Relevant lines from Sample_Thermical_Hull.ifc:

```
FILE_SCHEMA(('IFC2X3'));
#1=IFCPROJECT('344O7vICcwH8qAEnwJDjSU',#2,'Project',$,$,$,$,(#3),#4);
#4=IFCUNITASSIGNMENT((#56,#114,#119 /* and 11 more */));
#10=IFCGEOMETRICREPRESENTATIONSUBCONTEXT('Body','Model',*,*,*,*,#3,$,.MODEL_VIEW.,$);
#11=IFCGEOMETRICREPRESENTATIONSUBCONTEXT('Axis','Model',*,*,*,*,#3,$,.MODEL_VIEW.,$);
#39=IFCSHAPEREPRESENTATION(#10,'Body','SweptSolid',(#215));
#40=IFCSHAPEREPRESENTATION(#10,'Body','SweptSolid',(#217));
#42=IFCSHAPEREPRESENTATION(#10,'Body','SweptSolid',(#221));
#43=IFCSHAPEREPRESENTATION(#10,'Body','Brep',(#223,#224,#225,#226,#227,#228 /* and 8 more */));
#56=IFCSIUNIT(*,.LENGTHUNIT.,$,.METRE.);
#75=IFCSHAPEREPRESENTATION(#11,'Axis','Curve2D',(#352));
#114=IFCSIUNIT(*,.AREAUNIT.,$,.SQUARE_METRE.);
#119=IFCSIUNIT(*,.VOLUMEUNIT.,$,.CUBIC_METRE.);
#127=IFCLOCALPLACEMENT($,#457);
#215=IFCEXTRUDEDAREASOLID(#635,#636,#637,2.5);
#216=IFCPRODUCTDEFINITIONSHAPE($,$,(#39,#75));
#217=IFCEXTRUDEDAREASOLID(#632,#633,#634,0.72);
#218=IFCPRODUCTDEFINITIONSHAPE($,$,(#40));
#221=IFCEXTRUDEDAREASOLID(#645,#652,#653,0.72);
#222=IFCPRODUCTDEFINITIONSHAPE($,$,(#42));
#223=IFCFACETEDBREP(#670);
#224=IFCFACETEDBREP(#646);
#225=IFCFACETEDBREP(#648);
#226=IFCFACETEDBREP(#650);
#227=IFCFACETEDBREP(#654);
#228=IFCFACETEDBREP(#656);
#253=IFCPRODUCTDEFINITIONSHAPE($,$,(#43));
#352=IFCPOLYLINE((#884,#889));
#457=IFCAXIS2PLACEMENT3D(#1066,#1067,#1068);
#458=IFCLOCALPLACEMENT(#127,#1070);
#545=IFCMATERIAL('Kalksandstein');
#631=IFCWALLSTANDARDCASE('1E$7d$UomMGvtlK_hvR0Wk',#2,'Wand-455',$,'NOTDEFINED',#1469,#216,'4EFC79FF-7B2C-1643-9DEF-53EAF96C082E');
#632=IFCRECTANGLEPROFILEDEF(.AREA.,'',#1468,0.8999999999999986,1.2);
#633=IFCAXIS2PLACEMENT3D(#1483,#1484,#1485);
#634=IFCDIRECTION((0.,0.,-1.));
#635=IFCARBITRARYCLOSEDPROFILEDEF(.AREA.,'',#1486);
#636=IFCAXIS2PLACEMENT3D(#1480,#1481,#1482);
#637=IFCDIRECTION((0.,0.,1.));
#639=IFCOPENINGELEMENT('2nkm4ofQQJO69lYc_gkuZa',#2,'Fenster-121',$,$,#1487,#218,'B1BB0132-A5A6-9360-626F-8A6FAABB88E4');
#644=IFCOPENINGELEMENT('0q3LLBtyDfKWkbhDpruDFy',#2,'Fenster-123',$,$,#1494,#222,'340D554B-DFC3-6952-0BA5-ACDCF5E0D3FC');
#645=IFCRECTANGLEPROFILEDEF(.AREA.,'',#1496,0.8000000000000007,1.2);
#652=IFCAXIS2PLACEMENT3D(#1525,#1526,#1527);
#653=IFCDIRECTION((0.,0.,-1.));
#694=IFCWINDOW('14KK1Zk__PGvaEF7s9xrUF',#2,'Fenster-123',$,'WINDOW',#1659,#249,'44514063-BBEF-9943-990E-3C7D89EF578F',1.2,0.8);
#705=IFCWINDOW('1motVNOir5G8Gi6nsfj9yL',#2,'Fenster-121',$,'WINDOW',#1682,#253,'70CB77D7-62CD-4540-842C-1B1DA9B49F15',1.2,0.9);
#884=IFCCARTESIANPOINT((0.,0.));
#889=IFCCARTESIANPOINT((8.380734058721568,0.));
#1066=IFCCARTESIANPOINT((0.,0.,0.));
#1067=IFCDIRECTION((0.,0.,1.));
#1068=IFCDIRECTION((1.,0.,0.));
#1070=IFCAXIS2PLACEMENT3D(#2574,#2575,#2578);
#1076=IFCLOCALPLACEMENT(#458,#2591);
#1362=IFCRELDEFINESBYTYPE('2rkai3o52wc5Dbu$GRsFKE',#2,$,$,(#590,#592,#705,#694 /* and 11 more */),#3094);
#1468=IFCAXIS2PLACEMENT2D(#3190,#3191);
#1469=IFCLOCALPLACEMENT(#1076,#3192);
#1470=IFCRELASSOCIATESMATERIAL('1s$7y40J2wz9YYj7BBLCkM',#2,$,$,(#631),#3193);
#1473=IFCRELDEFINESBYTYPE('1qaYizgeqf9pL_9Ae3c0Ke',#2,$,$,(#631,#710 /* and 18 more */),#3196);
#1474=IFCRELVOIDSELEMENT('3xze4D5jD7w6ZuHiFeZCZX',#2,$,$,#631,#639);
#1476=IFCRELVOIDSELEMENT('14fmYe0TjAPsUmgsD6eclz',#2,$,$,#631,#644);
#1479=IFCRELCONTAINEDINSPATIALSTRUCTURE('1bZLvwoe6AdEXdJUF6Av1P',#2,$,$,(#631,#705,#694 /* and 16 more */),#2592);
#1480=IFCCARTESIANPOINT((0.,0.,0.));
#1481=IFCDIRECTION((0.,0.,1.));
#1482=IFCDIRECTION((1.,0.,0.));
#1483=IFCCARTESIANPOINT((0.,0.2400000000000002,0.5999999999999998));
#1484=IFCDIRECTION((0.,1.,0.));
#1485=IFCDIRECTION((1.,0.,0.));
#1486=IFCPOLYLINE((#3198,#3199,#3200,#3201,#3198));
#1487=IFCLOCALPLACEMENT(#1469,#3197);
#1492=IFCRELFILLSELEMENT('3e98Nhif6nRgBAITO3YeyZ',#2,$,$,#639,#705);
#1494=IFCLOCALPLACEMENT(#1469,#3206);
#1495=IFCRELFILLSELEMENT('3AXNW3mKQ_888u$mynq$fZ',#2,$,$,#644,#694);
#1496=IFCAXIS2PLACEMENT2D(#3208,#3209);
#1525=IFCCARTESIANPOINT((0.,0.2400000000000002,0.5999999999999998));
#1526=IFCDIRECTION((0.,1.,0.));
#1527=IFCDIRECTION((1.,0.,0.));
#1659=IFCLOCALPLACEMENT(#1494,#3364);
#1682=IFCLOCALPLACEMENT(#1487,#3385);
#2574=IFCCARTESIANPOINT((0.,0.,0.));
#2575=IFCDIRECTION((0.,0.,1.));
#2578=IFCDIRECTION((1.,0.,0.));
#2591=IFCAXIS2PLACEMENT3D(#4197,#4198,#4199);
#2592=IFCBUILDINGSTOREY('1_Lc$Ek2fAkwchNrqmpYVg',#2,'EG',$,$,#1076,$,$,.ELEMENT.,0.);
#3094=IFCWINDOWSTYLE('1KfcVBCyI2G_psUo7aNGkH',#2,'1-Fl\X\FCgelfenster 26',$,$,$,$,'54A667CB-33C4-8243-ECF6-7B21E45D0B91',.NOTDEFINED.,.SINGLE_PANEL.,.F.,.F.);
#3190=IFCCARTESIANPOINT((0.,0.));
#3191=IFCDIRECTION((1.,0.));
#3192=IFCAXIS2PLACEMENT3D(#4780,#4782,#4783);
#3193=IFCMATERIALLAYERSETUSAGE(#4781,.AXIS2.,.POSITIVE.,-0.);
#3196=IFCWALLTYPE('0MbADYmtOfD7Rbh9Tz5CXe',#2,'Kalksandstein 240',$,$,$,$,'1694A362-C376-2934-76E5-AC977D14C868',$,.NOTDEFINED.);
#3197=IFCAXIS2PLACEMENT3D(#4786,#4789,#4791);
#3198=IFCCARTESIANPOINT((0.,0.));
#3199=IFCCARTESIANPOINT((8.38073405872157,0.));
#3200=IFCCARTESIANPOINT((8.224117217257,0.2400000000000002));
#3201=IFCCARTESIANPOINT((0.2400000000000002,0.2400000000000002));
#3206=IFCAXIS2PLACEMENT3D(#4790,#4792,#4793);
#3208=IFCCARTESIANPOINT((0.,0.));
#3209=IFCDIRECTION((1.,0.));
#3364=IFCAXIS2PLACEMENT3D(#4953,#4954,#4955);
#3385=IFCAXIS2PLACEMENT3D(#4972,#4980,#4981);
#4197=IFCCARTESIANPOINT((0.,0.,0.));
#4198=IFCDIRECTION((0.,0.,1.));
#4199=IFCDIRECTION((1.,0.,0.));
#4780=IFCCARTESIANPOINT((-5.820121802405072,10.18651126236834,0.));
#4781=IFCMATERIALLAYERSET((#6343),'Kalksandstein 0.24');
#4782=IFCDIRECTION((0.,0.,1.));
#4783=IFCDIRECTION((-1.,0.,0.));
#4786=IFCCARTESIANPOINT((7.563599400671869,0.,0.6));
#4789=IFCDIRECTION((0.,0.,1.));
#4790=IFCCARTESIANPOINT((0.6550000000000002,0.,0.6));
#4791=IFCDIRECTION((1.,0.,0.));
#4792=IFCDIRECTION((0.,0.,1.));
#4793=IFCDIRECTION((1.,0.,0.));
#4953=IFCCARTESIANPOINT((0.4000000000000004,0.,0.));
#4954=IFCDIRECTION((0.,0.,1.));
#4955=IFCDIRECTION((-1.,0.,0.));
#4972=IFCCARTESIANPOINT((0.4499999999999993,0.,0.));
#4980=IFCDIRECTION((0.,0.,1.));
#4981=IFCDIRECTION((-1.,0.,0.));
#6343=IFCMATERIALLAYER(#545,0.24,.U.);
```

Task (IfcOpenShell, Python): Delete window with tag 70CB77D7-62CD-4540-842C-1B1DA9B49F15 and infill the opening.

```python
import ifcopenshell
import ifcopenshell.api.feature
import ifcopenshell.api.root
import ifcopenshell.geom
import ifcopenshell.util.shape

model = ifcopenshell.open("Sample_Thermical_Hull.ifc")
settings = ifcopenshell.geom.settings()


def volume(element):
    """Net volume in cubic metres, openings subtracted."""
    shape = ifcopenshell.geom.create_shape(settings, element)
    return ifcopenshell.util.shape.get_volume(shape.geometry)


window = model.by_guid("1motVNOir5G8Gi6nsfj9yL")
opening = window.FillsVoids[0].RelatingOpeningElement
wall = opening.VoidsElements[0].RelatingBuildingElement
before = volume(wall)

ifcopenshell.api.root.remove_product(model, product=window)
ifcopenshell.api.feature.remove_feature(model, feature=opening)

after = volume(wall)

print(f"wall volume {before:.3f} -> {after:.3f} m3")

model.write("Sample_Thermical_Hull_updated.ifc")
```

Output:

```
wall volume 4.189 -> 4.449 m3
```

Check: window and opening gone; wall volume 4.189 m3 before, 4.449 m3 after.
